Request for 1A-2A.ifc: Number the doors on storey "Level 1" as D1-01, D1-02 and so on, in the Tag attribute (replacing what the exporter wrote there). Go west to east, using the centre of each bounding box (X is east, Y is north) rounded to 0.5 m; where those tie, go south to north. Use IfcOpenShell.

First a look at what the model holds.

```python
import ifcopenshell
import ifcopenshell.util.element
import ifcopenshell.util.placement

model = ifcopenshell.open("1A-2A.ifc")
print(model.schema)
storey = next(s for s in model.by_type("IfcBuildingStorey") if s.Name == "Level 1")
doors = [e for e in ifcopenshell.util.element.get_decomposition(storey) if e.is_a("IfcDoor")]
for e in sorted(doors, key=lambda e: e.id()):
    origin = ifcopenshell.util.placement.get_local_placement(e.ObjectPlacement)[:3, 3]
    print(e.id(), e.Tag, e.Name, origin.round(2) + 0.0, sep=" | ")
```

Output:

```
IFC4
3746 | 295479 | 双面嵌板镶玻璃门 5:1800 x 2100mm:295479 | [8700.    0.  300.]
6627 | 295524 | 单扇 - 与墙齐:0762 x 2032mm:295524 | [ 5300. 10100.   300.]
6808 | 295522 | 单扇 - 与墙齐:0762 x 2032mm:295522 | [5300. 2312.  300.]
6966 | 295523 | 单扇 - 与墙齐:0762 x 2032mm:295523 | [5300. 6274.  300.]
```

```python
import ifcopenshell
import ifcopenshell.geom
import ifcopenshell.util.element
import ifcopenshell.util.shape

model = ifcopenshell.open("1A-2A.ifc")
settings = ifcopenshell.geom.settings()
settings.set("use-world-coords", True)


def centre(element):
    shape = ifcopenshell.geom.create_shape(settings, element)
    return ifcopenshell.util.shape.get_bbox_centroid(shape.geometry)


storey = next(s for s in model.by_type("IfcBuildingStorey") if s.Name == "Level 1")
doors = [e for e in ifcopenshell.util.element.get_decomposition(storey) if e.is_a("IfcDoor")]

# Insertion points can sit at a corner or the storey origin, so sort by the geometry (in metres).
centres = {e: centre(e) for e in doors}
doors.sort(key=lambda e: (round(centres[e][0] / 0.5), centres[e][1]))

for i, e in enumerate(doors, start=1):
    number = f"D1-{i:02d}"
    e.Tag = number
    print(e.id(), number)

model.write("1A-2A_updated.ifc")
```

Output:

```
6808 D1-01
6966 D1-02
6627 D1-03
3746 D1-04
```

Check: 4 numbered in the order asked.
